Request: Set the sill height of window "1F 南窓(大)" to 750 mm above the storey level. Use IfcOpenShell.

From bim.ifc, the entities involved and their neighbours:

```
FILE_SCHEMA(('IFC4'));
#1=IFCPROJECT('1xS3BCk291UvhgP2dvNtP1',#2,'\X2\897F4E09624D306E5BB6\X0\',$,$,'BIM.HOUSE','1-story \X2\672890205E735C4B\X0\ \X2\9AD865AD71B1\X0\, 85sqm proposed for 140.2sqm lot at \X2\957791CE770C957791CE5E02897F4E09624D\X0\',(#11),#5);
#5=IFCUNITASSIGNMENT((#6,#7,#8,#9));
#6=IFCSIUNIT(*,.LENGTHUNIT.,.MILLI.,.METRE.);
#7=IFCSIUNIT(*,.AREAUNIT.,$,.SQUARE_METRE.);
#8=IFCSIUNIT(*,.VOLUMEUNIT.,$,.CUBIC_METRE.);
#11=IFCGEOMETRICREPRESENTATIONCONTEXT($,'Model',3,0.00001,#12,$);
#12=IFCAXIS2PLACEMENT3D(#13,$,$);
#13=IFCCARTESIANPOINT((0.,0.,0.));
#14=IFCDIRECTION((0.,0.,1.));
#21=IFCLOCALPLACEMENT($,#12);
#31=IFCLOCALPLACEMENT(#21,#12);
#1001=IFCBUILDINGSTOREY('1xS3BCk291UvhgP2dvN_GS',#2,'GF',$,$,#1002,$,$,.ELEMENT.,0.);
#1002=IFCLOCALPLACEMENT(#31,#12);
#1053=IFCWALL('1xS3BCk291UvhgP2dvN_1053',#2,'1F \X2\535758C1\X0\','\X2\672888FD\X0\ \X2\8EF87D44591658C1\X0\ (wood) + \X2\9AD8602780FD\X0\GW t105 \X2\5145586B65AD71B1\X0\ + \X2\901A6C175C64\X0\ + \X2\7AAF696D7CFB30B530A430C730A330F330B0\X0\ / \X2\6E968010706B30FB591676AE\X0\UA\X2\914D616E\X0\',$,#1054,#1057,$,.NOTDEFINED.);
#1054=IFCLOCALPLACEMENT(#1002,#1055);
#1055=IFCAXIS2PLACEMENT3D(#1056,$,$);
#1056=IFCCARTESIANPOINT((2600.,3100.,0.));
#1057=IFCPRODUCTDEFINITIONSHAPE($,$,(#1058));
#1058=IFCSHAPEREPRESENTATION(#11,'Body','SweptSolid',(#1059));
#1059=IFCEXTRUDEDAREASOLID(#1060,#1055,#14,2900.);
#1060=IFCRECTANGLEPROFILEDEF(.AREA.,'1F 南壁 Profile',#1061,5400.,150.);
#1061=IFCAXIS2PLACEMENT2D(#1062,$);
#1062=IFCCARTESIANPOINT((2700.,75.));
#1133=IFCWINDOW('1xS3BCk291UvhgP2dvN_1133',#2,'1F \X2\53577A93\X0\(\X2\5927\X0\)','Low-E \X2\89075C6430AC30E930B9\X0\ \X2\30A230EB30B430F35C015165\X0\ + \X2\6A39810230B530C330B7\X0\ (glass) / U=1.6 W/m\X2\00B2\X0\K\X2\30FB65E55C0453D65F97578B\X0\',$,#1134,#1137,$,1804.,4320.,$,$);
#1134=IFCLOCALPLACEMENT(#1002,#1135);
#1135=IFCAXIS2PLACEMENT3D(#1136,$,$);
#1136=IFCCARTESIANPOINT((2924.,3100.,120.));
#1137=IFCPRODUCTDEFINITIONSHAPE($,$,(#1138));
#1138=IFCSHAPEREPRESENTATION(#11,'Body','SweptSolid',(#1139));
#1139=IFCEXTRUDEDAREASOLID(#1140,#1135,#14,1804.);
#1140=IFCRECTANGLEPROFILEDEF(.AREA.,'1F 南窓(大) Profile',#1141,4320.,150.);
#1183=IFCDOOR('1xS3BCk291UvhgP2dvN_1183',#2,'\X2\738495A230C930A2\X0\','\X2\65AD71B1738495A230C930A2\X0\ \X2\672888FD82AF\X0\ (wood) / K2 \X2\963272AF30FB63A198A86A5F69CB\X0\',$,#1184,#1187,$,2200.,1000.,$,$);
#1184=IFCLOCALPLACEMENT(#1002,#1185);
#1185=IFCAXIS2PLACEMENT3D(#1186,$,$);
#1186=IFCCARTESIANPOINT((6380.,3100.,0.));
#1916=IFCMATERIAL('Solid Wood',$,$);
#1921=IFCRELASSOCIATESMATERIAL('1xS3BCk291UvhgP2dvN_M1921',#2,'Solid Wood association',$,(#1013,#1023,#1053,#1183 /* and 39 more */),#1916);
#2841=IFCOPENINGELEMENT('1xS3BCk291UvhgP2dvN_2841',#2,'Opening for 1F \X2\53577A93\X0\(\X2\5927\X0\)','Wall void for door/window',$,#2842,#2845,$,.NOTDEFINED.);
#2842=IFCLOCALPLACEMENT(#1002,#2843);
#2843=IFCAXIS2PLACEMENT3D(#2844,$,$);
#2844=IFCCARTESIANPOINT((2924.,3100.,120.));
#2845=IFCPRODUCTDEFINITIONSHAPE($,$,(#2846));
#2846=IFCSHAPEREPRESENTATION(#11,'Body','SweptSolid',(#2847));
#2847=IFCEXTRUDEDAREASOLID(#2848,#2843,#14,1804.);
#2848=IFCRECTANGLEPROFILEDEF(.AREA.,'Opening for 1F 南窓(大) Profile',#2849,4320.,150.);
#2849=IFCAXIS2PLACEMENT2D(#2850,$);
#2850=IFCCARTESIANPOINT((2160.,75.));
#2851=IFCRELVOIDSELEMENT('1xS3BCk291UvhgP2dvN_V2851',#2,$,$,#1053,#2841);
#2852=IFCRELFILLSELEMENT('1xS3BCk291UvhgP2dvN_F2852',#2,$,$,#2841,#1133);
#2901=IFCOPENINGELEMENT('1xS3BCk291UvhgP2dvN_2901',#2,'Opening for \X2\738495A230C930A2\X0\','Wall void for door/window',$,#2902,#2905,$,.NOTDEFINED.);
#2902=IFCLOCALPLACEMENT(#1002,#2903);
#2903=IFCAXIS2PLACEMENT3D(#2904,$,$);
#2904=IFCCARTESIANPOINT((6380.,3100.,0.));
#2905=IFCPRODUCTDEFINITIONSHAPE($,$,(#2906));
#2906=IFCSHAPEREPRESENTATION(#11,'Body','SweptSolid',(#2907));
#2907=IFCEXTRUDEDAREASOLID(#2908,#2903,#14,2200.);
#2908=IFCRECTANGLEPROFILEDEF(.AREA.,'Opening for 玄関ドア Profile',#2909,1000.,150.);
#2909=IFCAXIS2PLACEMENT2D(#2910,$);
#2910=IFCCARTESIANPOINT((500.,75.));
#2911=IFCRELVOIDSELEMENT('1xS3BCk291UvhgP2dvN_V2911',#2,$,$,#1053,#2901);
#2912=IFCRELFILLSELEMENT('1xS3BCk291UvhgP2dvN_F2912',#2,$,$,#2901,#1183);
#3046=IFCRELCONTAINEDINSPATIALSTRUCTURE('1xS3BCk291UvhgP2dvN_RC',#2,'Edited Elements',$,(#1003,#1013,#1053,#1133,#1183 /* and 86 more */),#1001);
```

```python
import numpy as np
import ifcopenshell
import ifcopenshell.api.geometry
import ifcopenshell.geom
import ifcopenshell.util.element
import ifcopenshell.util.placement
import ifcopenshell.util.shape
import ifcopenshell.util.unit

model = ifcopenshell.open("bim.ifc")
unit_scale = ifcopenshell.util.unit.calculate_unit_scale(model)

window = model.by_id(1133)
opening = window.FillsVoids[0].RelatingOpeningElement
storey = ifcopenshell.util.element.get_container(window, ifc_class="IfcBuildingStorey")
level = ifcopenshell.util.placement.get_local_placement(storey.ObjectPlacement)[2, 3]

# The opening's origin need not be at the sill, so measure its lowest point.
shape = ifcopenshell.geom.create_shape(ifcopenshell.geom.settings(), opening)
bottom = ifcopenshell.util.shape.get_shape_bottom_elevation(shape, shape.geometry) / unit_scale
dz = level + 0.75 / unit_scale - bottom

shift = np.array([0.0, 0.0, dz])
# The window is not placed relative to its opening, so move both.
for product in (opening, window):
    matrix = ifcopenshell.util.placement.get_local_placement(product.ObjectPlacement)
    matrix[:3, 3] += shift
    ifcopenshell.api.geometry.edit_object_placement(model, product=product, matrix=matrix, is_si=False)

print(f"moved by {dz * unit_scale:+.3f} m")

model.write("bim_edited.ifc")
```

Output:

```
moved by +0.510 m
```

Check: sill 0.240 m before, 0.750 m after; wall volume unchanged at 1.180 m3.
